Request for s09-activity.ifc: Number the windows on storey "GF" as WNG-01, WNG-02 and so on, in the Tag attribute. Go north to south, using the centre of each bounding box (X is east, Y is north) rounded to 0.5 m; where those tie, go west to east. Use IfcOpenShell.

First a look at what the model holds.

```python
import ifcopenshell
import ifcopenshell.util.element
import ifcopenshell.util.placement

model = ifcopenshell.open("s09-activity.ifc")
print(model.schema)
storey = next(s for s in model.by_type("IfcBuildingStorey") if s.Name == "GF")
windows = [e for e in ifcopenshell.util.element.get_decomposition(storey) if e.is_a("IfcWindow")]
for e in sorted(windows, key=lambda e: e.id()):
    origin = ifcopenshell.util.placement.get_local_placement(e.ObjectPlacement)[:3, 3]
    print(e.id(), e.Tag, e.Name, origin.round(2) + 0.0, sep=" | ")
```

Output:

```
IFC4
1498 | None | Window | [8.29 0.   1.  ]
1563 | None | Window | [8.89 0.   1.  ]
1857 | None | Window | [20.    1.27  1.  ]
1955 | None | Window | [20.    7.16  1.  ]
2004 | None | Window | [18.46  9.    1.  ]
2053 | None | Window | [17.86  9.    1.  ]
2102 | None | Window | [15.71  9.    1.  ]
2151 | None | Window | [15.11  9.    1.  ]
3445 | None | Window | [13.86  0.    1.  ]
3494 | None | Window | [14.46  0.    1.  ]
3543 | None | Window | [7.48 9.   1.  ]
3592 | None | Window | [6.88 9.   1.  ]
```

```python
import ifcopenshell
import ifcopenshell.geom
import ifcopenshell.util.element
import ifcopenshell.util.shape

model = ifcopenshell.open("s09-activity.ifc")
settings = ifcopenshell.geom.settings()
settings.set("use-world-coords", True)


def centre(element):
    shape = ifcopenshell.geom.create_shape(settings, element)
    return ifcopenshell.util.shape.get_bbox_centroid(shape.geometry)


storey = next(s for s in model.by_type("IfcBuildingStorey") if s.Name == "GF")
windows = [e for e in ifcopenshell.util.element.get_decomposition(storey) if e.is_a("IfcWindow")]

# Insertion points can sit at a corner or the storey origin, so sort by the geometry (in metres).
centres = {e: centre(e) for e in windows}
windows.sort(key=lambda e: (-round(centres[e][1] / 0.5), centres[e][0]))

for i, e in enumerate(windows, start=1):
    number = f"WNG-{i:02d}"
    e.Tag = number
    print(e.id(), number)

model.write("s09-activity_v2.ifc")
```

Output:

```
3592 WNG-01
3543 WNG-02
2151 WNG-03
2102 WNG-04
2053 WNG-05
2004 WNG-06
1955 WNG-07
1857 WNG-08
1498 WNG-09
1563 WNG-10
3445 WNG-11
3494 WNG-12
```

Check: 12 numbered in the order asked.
